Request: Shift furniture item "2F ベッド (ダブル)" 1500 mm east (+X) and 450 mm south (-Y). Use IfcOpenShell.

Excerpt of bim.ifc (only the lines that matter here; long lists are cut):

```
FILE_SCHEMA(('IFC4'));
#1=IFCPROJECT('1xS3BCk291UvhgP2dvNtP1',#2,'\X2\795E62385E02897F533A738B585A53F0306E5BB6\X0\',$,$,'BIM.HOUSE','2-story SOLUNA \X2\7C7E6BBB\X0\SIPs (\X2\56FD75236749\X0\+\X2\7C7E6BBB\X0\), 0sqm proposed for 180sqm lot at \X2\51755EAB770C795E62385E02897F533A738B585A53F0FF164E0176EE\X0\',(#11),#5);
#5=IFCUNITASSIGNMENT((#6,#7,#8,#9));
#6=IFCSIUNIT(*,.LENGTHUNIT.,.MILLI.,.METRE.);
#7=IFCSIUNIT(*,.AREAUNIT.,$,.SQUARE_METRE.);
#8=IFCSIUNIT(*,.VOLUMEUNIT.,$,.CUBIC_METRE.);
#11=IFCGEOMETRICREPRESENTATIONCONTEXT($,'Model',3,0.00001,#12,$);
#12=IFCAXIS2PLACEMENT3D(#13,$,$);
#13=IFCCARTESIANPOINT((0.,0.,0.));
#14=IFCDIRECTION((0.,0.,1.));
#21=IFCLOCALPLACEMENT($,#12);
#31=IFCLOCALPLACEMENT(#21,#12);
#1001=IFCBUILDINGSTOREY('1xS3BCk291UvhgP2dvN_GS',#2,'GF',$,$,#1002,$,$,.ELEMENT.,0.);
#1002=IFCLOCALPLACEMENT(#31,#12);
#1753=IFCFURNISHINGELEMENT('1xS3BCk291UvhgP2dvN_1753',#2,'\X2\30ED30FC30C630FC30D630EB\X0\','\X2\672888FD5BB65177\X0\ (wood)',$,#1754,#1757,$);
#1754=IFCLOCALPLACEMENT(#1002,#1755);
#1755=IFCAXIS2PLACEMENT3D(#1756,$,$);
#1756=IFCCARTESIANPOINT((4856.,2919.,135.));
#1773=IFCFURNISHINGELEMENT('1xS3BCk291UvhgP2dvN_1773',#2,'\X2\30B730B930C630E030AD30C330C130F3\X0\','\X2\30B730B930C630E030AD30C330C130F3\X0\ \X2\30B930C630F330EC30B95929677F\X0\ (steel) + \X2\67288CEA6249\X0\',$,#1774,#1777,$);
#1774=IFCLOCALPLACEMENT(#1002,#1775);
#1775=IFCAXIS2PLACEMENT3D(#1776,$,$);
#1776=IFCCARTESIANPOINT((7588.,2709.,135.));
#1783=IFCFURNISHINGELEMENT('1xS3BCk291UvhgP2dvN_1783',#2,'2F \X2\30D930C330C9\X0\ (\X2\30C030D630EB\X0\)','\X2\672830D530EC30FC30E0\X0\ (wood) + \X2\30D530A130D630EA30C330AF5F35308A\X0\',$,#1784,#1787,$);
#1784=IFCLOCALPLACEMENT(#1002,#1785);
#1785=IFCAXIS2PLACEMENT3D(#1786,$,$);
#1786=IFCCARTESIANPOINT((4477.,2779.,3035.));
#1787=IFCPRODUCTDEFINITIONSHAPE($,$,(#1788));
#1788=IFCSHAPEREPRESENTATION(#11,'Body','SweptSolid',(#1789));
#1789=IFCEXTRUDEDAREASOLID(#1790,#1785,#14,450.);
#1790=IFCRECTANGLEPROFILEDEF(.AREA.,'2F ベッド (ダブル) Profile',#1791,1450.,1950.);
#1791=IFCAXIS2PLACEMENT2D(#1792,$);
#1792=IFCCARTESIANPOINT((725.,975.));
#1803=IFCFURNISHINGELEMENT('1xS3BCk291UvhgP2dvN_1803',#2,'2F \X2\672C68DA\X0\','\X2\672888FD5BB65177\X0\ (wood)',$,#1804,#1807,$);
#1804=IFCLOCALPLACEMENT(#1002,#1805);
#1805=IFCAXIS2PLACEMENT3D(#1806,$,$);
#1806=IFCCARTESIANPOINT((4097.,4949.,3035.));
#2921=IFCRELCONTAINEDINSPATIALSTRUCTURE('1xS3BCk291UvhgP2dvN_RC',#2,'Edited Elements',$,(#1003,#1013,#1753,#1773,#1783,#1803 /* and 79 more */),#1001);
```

```python
import ifcopenshell
import ifcopenshell.api.geometry
import ifcopenshell.util.placement
import ifcopenshell.util.unit

model = ifcopenshell.open("bim.ifc")
unit_scale = ifcopenshell.util.unit.calculate_unit_scale(model)

item = model.by_id(1783)
matrix = ifcopenshell.util.placement.get_local_placement(item.ObjectPlacement)
matrix[0, 3] += 1.5 / unit_scale
matrix[1, 3] -= 0.45 / unit_scale
ifcopenshell.api.geometry.edit_object_placement(model, product=item, matrix=matrix, is_si=False)

print(ifcopenshell.util.placement.get_local_placement(item.ObjectPlacement).round(3) + 0.0)

model.write("bim_rev.ifc")
```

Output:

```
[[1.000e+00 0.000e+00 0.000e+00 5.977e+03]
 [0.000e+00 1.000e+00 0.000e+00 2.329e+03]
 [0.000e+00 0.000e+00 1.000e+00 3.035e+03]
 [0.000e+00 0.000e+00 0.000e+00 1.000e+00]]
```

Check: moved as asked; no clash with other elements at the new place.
